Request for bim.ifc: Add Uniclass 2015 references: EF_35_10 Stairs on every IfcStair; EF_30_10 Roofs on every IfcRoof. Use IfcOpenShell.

First a look at what the model holds.

```python
import ifcopenshell

model = ifcopenshell.open("bim.ifc")
print(model.schema)
print("classifications:", [c.Name for c in model.by_type("IfcClassification")])
for ifc_class in ("IfcDoor", "IfcRoof", "IfcStair", "IfcWall", "IfcWindow"):
    print(ifc_class, len(model.by_type(ifc_class)))
```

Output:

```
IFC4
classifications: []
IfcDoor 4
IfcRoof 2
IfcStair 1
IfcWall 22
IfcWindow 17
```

```python
import ifcopenshell
import ifcopenshell.api.classification

model = ifcopenshell.open("bim.ifc")

system = ifcopenshell.api.classification.add_classification(model, classification="Uniclass 2015")

codes = {
    "IfcStair": ("EF_35_10", "Stairs"),
    "IfcRoof": ("EF_30_10", "Roofs"),
}
for ifc_class, (code, name) in codes.items():
    products = model.by_type(ifc_class)
    ifcopenshell.api.classification.add_reference(
        model, products=products, classification=system, identification=code, name=name
    )
    print(code, len(products))

model.write("bim_edited.ifc")
```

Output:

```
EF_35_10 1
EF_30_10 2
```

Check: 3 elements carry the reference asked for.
